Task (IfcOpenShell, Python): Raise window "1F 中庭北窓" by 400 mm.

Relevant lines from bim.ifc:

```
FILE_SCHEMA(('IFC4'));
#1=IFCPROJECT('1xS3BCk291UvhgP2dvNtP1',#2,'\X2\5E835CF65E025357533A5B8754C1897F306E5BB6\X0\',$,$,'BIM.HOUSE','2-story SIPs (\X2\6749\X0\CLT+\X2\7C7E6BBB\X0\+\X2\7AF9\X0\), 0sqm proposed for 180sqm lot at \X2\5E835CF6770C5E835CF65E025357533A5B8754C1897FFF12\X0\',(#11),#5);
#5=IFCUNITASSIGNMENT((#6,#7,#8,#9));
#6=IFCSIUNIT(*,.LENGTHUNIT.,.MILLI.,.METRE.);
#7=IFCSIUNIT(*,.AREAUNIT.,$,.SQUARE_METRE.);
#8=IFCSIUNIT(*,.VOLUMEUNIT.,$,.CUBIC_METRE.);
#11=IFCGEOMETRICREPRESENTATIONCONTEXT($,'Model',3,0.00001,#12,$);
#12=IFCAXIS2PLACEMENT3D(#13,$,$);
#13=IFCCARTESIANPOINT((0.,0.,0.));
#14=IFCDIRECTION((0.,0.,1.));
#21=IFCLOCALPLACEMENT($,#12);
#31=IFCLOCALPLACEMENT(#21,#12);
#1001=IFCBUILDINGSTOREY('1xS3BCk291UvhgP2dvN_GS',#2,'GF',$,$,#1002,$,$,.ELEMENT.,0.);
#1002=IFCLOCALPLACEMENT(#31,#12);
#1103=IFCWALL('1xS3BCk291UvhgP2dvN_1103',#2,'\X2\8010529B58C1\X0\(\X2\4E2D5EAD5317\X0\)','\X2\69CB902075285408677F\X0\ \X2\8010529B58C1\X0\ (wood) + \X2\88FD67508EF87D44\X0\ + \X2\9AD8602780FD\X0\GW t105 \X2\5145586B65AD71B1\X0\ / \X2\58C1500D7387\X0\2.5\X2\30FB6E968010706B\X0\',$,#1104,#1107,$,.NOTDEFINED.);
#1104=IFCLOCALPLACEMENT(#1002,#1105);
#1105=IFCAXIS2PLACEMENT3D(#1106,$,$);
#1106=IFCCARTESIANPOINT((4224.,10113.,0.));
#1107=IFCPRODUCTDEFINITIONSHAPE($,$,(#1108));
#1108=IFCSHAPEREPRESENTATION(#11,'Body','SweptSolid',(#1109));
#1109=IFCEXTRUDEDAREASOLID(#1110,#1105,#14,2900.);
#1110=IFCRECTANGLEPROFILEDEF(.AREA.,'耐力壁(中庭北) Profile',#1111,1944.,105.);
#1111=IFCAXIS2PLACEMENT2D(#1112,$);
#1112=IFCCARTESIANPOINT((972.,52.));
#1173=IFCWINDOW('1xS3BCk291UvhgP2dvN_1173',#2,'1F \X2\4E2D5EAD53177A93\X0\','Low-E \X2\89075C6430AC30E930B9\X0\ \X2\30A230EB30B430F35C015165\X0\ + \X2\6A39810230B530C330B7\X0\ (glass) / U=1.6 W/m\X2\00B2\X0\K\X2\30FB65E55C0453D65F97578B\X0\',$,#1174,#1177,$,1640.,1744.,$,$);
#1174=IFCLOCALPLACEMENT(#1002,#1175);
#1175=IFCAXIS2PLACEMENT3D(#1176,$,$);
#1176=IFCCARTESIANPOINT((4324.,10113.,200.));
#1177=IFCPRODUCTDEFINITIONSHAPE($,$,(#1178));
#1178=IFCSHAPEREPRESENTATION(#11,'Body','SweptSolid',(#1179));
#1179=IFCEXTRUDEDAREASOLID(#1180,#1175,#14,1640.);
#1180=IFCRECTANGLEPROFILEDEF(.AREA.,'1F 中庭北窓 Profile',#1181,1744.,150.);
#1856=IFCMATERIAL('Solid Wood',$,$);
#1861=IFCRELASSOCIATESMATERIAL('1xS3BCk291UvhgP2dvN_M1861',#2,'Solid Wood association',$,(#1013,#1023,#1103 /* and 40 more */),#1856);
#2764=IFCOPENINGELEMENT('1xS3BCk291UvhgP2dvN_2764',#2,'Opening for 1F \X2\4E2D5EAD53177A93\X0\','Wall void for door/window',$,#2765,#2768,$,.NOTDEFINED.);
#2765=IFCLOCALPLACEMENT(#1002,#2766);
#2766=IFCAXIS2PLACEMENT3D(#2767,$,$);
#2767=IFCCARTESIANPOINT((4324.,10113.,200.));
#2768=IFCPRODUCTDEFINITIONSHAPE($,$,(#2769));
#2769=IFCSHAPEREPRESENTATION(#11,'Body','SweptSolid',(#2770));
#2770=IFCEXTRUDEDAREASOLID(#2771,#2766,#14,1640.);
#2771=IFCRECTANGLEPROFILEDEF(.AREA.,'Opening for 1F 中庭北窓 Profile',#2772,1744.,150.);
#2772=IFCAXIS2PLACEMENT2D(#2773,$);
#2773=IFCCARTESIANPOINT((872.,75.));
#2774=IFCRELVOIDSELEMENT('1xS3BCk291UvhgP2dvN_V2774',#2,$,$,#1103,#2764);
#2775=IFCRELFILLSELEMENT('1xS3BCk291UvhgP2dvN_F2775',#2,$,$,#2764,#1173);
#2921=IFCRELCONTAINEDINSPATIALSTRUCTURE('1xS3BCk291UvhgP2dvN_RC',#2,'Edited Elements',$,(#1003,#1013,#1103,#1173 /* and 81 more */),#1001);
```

```python
import numpy as np
import ifcopenshell
import ifcopenshell.api.geometry
import ifcopenshell.util.placement
import ifcopenshell.util.unit

model = ifcopenshell.open("bim.ifc")
unit_scale = ifcopenshell.util.unit.calculate_unit_scale(model)

window = model.by_guid("1xS3BCk291UvhgP2dvN_1173")
opening = window.FillsVoids[0].RelatingOpeningElement
dz = 400.0

shift = np.array([0.0, 0.0, dz])
# The window is not placed relative to its opening, so move both.
for product in (opening, window):
    matrix = ifcopenshell.util.placement.get_local_placement(product.ObjectPlacement)
    matrix[:3, 3] += shift
    ifcopenshell.api.geometry.edit_object_placement(model, product=product, matrix=matrix, is_si=False)

print(f"moved by {dz * unit_scale:+.3f} m")

model.write("bim-out.ifc")
```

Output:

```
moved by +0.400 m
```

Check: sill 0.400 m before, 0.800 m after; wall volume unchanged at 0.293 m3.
